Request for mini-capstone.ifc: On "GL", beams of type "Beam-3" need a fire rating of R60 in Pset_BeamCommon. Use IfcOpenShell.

First a look at what the model holds.

```python
import ifcopenshell
import ifcopenshell.util.element

model = ifcopenshell.open("mini-capstone.ifc")
print(model.schema)
storey = next(s for s in model.by_type("IfcBuildingStorey") if s.Name == "GL")
beams = [e for e in ifcopenshell.util.element.get_decomposition(storey) if e.is_a("IfcBeam")]
seen = {}
for e in beams:
    element_type = ifcopenshell.util.element.get_type(e)
    key = (element_type.Name if element_type != e and element_type else None, ifcopenshell.util.element.get_pset(e, "Pset_BeamCommon", "FireRating"))
    seen[key] = seen.get(key, 0) + 1
for (name, value), count in sorted(seen.items(), key=str):
    print(count, "x", name, "|", value)
```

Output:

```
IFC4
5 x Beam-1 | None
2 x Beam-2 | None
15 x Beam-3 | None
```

```python
import ifcopenshell
import ifcopenshell.api.pset
import ifcopenshell.util.element

model = ifcopenshell.open("mini-capstone.ifc")

storey = next(s for s in model.by_type("IfcBuildingStorey") if s.Name == "GL")
beams = [e for e in ifcopenshell.util.element.get_decomposition(storey) if e.is_a("IfcBeam")]

count = 0
for e in beams:
    element_type = ifcopenshell.util.element.get_type(e)
    if element_type in (None, e) or element_type.Name != "Beam-3":
        continue
    # add_pset returns the element's existing set when there is one.
    pset = ifcopenshell.api.pset.add_pset(model, product=e, name="Pset_BeamCommon")
    ifcopenshell.api.pset.edit_pset(model, pset=pset, properties={"FireRating": "R60"})
    count += 1

print(count, "beams updated")

model.write("mini-capstone_v2.ifc")
```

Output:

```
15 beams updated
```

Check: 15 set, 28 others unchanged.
